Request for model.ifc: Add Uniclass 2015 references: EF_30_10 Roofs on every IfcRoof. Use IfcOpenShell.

First a look at what the model holds.

```python
import ifcopenshell

model = ifcopenshell.open("model.ifc")
print(model.schema)
print("classifications:", [c.Name for c in model.by_type("IfcClassification")])
for ifc_class in ("IfcDoor", "IfcRoof", "IfcStair", "IfcWall", "IfcWindow"):
    print(ifc_class, len(model.by_type(ifc_class)))
```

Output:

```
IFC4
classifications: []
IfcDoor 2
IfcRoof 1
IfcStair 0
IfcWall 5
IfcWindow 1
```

```python
import ifcopenshell
import ifcopenshell.api.classification

model = ifcopenshell.open("model.ifc")

system = ifcopenshell.api.classification.add_classification(model, classification="Uniclass 2015")

codes = {
    "IfcRoof": ("EF_30_10", "Roofs"),
}
for ifc_class, (code, name) in codes.items():
    products = model.by_type(ifc_class)
    ifcopenshell.api.classification.add_reference(
        model, products=products, classification=system, identification=code, name=name
    )
    print(code, len(products))

model.write("model_updated.ifc")
```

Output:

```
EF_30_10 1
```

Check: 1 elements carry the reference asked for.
